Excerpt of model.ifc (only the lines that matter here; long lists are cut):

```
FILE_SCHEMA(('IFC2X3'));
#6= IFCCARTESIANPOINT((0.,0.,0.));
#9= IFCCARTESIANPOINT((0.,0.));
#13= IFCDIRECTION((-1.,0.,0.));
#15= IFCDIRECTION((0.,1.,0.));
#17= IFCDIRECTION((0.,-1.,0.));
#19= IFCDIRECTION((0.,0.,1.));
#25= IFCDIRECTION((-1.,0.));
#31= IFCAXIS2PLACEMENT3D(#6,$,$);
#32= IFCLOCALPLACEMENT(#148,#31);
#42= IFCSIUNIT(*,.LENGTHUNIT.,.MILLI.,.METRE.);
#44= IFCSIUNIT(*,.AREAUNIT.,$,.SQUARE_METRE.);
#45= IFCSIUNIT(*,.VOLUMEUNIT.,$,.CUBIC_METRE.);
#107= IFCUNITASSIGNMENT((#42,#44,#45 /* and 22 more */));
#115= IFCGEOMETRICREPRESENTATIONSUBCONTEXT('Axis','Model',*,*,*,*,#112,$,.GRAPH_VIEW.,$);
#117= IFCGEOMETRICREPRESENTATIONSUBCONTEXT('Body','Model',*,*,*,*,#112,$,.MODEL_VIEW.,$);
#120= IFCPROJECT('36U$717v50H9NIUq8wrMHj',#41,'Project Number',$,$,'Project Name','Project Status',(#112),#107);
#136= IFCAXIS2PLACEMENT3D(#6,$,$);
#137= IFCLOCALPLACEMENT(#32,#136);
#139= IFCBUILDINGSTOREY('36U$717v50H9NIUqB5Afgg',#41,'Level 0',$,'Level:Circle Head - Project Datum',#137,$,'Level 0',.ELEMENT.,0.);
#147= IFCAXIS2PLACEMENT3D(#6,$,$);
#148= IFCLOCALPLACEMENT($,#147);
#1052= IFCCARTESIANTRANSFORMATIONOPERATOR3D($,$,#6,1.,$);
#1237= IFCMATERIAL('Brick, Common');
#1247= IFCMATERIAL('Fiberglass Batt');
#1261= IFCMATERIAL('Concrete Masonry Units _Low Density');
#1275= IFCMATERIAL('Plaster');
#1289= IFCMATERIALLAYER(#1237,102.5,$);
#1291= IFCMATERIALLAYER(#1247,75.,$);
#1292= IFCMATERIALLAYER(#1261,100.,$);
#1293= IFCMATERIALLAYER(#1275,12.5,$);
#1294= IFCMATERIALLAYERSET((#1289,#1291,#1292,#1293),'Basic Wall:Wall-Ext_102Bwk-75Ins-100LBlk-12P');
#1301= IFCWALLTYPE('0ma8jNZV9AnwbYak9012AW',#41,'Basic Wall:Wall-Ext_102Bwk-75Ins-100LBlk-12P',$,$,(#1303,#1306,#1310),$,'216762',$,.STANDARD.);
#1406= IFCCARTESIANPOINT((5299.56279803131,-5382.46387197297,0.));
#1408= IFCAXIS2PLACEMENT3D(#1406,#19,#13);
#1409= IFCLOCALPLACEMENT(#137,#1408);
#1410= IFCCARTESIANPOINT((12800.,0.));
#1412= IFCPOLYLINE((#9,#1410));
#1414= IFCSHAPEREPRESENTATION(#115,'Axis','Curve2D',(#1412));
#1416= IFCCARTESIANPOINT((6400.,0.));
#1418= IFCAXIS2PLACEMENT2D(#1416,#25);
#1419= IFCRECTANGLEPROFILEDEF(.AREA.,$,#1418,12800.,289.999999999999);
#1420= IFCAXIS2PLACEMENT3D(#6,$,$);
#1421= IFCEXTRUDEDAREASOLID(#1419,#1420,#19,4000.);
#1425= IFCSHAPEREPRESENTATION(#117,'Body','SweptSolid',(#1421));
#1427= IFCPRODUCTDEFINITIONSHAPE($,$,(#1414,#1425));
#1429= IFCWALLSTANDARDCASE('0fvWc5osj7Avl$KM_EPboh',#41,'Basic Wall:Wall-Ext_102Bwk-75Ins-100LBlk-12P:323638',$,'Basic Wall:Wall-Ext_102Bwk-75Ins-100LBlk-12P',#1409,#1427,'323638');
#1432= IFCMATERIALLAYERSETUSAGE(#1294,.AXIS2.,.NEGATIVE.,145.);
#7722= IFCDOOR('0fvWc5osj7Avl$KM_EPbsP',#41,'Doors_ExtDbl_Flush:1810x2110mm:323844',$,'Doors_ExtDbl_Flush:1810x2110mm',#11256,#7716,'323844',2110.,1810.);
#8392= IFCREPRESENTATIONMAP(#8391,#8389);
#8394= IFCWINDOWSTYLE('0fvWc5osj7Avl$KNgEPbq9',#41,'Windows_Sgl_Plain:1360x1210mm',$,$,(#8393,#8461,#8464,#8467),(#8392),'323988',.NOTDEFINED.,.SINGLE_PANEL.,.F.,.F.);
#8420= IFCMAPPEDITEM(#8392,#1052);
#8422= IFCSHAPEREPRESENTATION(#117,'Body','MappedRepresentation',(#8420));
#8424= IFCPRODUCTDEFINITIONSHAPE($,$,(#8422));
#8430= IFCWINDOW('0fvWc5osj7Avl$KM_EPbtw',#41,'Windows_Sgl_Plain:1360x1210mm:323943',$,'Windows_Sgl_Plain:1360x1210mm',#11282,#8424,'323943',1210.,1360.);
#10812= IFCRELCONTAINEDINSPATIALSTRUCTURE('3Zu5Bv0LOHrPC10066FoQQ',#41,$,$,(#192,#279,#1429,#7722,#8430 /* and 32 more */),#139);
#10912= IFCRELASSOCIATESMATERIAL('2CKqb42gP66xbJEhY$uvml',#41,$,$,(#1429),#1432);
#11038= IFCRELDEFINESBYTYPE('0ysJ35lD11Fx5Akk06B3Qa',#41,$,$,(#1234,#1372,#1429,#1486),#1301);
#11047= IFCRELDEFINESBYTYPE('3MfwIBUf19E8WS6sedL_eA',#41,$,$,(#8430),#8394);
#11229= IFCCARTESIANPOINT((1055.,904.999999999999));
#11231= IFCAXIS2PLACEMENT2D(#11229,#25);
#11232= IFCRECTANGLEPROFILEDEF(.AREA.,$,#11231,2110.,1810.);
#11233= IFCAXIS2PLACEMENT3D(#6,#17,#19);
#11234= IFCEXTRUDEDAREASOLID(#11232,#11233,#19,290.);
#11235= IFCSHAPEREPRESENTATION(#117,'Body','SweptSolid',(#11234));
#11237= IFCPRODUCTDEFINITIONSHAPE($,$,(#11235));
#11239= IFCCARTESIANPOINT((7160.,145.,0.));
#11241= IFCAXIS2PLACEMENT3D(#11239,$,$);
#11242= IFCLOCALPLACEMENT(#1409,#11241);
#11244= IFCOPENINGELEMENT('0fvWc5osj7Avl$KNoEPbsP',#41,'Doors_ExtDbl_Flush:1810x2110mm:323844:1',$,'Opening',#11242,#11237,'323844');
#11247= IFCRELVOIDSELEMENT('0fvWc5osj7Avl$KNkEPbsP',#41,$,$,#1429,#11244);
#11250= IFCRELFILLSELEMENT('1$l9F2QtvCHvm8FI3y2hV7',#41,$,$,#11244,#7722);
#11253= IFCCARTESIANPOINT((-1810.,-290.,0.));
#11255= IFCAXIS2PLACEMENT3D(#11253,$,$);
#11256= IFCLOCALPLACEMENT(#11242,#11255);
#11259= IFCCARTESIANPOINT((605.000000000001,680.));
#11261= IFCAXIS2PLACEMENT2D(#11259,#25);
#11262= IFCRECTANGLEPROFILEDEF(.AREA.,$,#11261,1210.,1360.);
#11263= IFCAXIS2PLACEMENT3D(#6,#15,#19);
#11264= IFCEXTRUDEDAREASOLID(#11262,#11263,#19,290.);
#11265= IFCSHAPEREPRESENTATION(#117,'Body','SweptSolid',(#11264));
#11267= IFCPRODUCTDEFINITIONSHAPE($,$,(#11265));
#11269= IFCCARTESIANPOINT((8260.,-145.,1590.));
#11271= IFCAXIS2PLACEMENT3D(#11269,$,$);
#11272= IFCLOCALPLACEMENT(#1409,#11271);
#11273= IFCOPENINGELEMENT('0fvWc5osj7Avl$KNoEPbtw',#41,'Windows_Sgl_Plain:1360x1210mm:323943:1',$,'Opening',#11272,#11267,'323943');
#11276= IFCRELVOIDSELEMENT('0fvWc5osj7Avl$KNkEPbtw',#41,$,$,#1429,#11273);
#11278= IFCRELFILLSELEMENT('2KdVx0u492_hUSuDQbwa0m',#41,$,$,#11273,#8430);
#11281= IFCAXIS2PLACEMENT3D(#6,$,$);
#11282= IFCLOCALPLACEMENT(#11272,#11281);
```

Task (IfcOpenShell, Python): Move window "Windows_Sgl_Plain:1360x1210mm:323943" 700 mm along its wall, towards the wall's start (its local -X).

```python
import ifcopenshell
import ifcopenshell.api.geometry
import ifcopenshell.util.placement
import ifcopenshell.util.unit

model = ifcopenshell.open("model.ifc")
unit_scale = ifcopenshell.util.unit.calculate_unit_scale(model)

window = model.by_guid("0fvWc5osj7Avl$KM_EPbtw")
opening = window.FillsVoids[0].RelatingOpeningElement
wall = opening.VoidsElements[0].RelatingBuildingElement

wall_matrix = ifcopenshell.util.placement.get_local_placement(wall.ObjectPlacement)
shift = wall_matrix[:3, 0] * -0.7 / unit_scale
before = ifcopenshell.util.placement.get_local_placement(window.ObjectPlacement)[:3, 3].copy()

# The window is placed relative to its opening, so it follows when the opening moves.
matrix = ifcopenshell.util.placement.get_local_placement(opening.ObjectPlacement)
matrix[:3, 3] += shift
ifcopenshell.api.geometry.edit_object_placement(
    model, product=opening, matrix=matrix, is_si=False, should_transform_children=True
)

after = ifcopenshell.util.placement.get_local_placement(window.ObjectPlacement)[:3, 3]
print("window moved by", (after - before).round(3) + 0.0)

model.write("model_edited.ifc")
```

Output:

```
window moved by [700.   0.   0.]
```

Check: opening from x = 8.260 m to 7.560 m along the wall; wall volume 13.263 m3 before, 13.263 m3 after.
